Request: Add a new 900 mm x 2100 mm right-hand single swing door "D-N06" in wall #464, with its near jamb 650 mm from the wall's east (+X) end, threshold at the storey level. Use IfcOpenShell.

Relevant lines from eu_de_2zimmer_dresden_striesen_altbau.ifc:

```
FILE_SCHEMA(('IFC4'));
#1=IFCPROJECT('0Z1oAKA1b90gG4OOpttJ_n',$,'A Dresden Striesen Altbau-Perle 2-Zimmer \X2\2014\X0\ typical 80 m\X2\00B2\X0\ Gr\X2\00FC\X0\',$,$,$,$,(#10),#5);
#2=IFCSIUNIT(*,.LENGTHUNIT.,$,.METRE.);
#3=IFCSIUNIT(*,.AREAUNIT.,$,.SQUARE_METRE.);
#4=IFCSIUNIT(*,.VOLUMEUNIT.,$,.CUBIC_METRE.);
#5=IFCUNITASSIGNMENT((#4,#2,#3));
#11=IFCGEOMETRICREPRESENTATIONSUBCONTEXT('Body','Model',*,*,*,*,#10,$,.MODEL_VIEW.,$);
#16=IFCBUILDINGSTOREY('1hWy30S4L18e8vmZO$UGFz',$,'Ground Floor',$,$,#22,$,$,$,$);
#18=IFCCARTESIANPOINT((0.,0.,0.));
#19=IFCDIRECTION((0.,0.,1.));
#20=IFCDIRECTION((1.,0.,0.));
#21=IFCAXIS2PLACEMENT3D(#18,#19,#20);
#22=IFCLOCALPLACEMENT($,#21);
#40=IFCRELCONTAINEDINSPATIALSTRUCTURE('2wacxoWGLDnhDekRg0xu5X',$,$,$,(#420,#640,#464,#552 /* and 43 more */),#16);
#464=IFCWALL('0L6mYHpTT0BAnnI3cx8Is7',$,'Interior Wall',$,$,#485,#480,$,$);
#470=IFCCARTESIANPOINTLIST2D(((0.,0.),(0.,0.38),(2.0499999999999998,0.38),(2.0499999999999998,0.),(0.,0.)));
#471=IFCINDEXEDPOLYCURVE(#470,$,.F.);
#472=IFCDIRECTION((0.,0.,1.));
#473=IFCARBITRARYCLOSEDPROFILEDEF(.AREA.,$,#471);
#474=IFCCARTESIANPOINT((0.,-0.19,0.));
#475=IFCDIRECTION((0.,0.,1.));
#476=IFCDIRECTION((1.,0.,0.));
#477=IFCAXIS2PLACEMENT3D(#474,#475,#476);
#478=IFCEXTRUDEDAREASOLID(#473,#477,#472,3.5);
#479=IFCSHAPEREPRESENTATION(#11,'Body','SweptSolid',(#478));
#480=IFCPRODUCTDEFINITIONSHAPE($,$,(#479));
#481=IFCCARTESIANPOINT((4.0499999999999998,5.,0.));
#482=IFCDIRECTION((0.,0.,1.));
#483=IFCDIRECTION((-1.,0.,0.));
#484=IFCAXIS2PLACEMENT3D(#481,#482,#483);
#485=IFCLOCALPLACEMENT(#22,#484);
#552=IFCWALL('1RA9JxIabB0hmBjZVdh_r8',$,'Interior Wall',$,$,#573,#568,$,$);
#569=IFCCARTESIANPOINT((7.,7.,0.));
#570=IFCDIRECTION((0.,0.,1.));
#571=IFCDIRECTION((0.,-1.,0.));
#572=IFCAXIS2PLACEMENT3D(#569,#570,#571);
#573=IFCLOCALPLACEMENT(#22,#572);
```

```python
import numpy as np
import ifcopenshell
import ifcopenshell.api.feature
import ifcopenshell.api.geometry
import ifcopenshell.api.root
import ifcopenshell.api.spatial
import ifcopenshell.geom
import ifcopenshell.util.element
import ifcopenshell.util.placement
import ifcopenshell.util.representation
import ifcopenshell.util.shape
import ifcopenshell.util.unit

model = ifcopenshell.open("eu_de_2zimmer_dresden_striesen_altbau.ifc")
unit_scale = ifcopenshell.util.unit.calculate_unit_scale(model)
settings = ifcopenshell.geom.settings()


def volume(element):
    """Net volume in cubic metres, openings subtracted."""
    shape = ifcopenshell.geom.create_shape(settings, element)
    return ifcopenshell.util.shape.get_volume(shape.geometry)


wall = model.by_guid("0L6mYHpTT0BAnnI3cx8Is7")
storey = ifcopenshell.util.element.get_container(wall, ifc_class="IfcBuildingStorey")
context = ifcopenshell.util.representation.get_context(model, "Model", "Body", "MODEL_VIEW")
before = volume(wall)

width, height, from_end, sill = 0.9, 2.1, 0.65, 0.0  # metres

# The wall runs along its own X axis, and the end named is its -X end.
wall_shape = ifcopenshell.geom.create_shape(settings, wall)
x, y, z = ifcopenshell.util.shape.get_vertices(wall_shape.geometry).T
start = x.min() + from_end
face, thickness = float(y.min()), float(y.max() - y.min())
wall_matrix = ifcopenshell.util.placement.get_local_placement(wall.ObjectPlacement)
level = ifcopenshell.util.placement.get_local_placement(storey.ObjectPlacement)[2, 3]


def in_wall(x, y):
    """Placement at x, y metres in the wall's axes, at sill height."""
    matrix = wall_matrix.copy()
    matrix[:, 3] = wall_matrix @ np.array([x / unit_scale, y / unit_scale, 0.0, 1.0])
    matrix[2, 3] = level + sill / unit_scale
    return matrix


# Opening: a box that overshoots both wall faces by 50 mm.
opening = ifcopenshell.api.root.create_entity(model, ifc_class="IfcOpeningElement", predefined_type="OPENING")
box = ifcopenshell.api.geometry.add_wall_representation(
    model, context=context, length=width, height=height, thickness=thickness + 0.1
)
ifcopenshell.api.geometry.assign_representation(model, product=opening, representation=box)
ifcopenshell.api.geometry.edit_object_placement(model, product=opening, matrix=in_wall(start, face - 0.05), is_si=False)
ifcopenshell.api.feature.add_feature(model, feature=opening, element=wall)

door = ifcopenshell.api.root.create_entity(model, ifc_class="IfcDoor", name="D-N06", predefined_type="DOOR")
door.OverallWidth, door.OverallHeight = width / unit_scale, height / unit_scale
door.OperationType = "SINGLE_SWING_RIGHT"
body = ifcopenshell.api.geometry.add_door_representation(
    model,
    context=context,
    overall_width=door.OverallWidth,
    overall_height=door.OverallHeight,
    operation_type="SINGLE_SWING_RIGHT",
    lining_properties={"LiningDepth": thickness / unit_scale, "ThresholdDepth": thickness / unit_scale},
)
ifcopenshell.api.geometry.assign_representation(model, product=door, representation=body)
ifcopenshell.api.spatial.assign_container(model, products=[door], relating_structure=storey)
ifcopenshell.api.feature.add_filling(model, opening=opening, element=door)

# The lining spans the wall, so the door starts at the wall face.
ifcopenshell.api.geometry.edit_object_placement(model, product=door, matrix=in_wall(start, face), is_si=False)

after = volume(wall)

print(f"wall volume {before:.3f} -> {after:.3f} m3")

model.write("eu_de_2zimmer_dresden_striesen_altbau_edited.ifc")
```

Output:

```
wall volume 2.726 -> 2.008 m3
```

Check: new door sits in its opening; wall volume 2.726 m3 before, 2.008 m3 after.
